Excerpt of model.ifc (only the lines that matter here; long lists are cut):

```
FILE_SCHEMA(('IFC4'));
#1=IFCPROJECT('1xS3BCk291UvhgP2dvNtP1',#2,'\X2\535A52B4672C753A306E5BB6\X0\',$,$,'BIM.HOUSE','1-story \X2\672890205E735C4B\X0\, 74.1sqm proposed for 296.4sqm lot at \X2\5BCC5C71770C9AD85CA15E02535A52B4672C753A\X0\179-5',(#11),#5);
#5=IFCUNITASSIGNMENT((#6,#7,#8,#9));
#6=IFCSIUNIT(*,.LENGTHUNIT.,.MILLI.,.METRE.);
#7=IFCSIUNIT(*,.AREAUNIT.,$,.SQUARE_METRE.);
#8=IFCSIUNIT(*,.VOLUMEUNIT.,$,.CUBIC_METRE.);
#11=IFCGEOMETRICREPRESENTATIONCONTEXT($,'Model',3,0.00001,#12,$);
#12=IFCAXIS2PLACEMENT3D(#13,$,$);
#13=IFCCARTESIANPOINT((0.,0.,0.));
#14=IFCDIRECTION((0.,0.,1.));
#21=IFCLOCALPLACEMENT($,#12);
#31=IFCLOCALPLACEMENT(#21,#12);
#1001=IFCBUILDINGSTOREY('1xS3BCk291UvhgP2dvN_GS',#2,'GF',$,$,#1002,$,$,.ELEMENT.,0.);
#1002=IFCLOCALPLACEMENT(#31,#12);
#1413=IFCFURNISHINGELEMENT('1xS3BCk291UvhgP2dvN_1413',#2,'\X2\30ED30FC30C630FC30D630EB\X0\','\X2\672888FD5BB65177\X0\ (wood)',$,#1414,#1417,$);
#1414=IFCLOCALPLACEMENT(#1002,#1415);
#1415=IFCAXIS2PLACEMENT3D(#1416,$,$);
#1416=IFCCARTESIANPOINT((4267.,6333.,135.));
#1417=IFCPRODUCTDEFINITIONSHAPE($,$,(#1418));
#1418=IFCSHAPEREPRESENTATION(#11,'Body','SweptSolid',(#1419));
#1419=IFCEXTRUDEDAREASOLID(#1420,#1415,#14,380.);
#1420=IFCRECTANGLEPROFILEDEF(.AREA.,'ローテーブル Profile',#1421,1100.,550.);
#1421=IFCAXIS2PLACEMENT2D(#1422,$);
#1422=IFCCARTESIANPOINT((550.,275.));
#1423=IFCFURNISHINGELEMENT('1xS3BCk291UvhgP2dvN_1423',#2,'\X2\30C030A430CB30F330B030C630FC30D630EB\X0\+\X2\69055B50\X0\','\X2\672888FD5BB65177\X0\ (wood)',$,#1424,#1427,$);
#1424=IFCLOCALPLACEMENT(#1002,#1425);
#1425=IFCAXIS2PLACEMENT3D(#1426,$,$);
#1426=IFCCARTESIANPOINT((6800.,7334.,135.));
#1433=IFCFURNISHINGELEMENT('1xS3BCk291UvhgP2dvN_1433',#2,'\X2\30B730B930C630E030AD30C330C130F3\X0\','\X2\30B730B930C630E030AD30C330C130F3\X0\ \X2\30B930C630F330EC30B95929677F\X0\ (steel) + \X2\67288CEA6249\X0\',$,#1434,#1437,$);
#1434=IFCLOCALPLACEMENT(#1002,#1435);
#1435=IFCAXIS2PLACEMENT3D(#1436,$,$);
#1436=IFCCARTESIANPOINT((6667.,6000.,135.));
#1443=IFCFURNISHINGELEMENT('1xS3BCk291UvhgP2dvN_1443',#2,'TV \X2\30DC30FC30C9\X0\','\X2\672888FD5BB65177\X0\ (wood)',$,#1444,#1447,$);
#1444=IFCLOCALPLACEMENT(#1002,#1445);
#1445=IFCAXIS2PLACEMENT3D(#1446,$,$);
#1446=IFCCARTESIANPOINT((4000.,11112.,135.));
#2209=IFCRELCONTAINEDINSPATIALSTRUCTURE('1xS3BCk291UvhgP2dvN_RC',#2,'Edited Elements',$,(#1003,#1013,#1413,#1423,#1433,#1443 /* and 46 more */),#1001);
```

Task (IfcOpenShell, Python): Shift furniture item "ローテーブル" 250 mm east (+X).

```python
import ifcopenshell
import ifcopenshell.api.geometry
import ifcopenshell.util.placement

model = ifcopenshell.open("model.ifc")

item = model.by_id(1413)
matrix = ifcopenshell.util.placement.get_local_placement(item.ObjectPlacement)
matrix[0, 3] += 250.0
ifcopenshell.api.geometry.edit_object_placement(model, product=item, matrix=matrix, is_si=False)

print(ifcopenshell.util.placement.get_local_placement(item.ObjectPlacement).round(3) + 0.0)

model.write("model_v2.ifc")
```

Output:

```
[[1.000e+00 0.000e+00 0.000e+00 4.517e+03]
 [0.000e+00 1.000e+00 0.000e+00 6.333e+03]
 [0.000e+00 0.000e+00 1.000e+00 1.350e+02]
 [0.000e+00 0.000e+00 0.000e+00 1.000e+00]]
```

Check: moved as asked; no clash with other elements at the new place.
